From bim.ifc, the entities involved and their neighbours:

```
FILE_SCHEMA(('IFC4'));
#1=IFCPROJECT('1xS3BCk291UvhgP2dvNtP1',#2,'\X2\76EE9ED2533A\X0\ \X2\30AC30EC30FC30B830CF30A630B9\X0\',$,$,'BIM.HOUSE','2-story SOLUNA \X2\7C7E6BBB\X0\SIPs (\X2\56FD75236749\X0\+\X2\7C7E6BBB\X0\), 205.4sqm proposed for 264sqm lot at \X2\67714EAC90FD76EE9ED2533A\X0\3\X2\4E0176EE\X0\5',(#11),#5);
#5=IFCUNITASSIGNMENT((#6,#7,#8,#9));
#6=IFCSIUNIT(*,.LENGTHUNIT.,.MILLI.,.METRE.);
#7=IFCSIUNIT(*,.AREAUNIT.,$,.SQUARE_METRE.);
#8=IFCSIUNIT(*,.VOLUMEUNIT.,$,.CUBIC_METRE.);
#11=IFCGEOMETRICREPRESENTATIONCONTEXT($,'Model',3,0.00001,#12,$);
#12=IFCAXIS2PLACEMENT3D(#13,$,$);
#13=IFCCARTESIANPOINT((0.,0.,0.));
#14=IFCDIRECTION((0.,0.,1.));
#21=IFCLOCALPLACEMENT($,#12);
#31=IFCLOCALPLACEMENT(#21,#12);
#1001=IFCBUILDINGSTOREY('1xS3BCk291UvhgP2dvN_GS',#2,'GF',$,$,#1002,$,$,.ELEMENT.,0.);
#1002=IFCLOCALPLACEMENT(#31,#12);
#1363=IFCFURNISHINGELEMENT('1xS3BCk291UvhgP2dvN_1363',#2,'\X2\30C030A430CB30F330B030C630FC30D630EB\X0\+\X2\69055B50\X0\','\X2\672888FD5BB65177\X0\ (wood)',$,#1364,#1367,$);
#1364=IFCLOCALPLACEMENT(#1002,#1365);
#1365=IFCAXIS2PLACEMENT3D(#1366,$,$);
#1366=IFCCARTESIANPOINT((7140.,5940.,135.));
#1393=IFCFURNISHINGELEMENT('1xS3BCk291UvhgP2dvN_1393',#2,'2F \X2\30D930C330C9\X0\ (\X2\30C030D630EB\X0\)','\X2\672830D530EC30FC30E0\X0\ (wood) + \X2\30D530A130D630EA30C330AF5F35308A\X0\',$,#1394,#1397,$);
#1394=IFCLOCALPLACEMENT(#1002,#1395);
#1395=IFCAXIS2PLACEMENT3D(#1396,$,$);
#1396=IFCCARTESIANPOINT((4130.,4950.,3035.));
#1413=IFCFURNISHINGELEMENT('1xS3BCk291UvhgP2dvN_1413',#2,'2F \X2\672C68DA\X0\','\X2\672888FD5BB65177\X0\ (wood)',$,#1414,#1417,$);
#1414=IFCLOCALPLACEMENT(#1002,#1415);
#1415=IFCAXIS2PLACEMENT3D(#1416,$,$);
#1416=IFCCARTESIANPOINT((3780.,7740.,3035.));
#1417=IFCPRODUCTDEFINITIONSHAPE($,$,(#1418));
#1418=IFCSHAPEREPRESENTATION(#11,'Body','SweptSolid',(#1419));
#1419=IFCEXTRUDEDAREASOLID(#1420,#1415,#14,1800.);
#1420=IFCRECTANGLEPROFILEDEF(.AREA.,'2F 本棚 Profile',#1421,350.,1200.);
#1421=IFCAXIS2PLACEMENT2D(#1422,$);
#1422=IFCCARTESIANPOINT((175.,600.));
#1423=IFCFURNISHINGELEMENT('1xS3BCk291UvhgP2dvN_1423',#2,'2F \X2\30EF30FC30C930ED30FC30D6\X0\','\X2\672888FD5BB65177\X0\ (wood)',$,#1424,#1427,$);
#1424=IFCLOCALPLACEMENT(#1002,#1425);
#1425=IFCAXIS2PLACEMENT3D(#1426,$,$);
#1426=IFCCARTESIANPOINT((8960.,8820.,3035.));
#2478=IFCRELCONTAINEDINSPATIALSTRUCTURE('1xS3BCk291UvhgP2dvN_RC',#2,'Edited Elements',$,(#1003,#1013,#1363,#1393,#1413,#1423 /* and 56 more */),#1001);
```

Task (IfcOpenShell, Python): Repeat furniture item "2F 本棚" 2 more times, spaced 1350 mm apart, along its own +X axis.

```python
import ifcopenshell
import ifcopenshell.api.geometry
import ifcopenshell.api.root
import ifcopenshell.util.element
import ifcopenshell.util.placement
import ifcopenshell.util.unit

model = ifcopenshell.open("bim.ifc")
unit_scale = ifcopenshell.util.unit.calculate_unit_scale(model)


def reuse_history(source, copy):
    """copy_class also copies each property set's owner history, people and application; keep the originals."""
    for rel in copy.IsDefinedBy:
        if rel.is_a("IfcRelDefinesByProperties") and (history := rel.RelatingPropertyDefinition.OwnerHistory):
            rel.RelatingPropertyDefinition.OwnerHistory = source.OwnerHistory
            ifcopenshell.util.element.remove_deep2(model, history)


source = model.by_guid("1xS3BCk291UvhgP2dvN_1413")
base = ifcopenshell.util.placement.get_local_placement(source.ObjectPlacement)
step = base[:3, 0] * 1.35 / unit_scale

for i in range(1, 3):
    copy = ifcopenshell.api.root.copy_class(model, product=source)
    copy.Representation = ifcopenshell.util.element.copy_deep(
        model, source.Representation, exclude=["IfcGeometricRepresentationContext", "IfcRepresentationMap"]
    )
    reuse_history(source, copy)
    matrix = base.copy()
    matrix[:3, 3] += i * step
    print("added at", matrix[:3, 3].round(3) + 0.0)
    ifcopenshell.api.geometry.edit_object_placement(model, product=copy, matrix=matrix, is_si=False)

model.write("bim_edited.ifc")
```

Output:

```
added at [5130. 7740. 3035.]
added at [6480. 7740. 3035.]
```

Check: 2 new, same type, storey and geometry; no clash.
